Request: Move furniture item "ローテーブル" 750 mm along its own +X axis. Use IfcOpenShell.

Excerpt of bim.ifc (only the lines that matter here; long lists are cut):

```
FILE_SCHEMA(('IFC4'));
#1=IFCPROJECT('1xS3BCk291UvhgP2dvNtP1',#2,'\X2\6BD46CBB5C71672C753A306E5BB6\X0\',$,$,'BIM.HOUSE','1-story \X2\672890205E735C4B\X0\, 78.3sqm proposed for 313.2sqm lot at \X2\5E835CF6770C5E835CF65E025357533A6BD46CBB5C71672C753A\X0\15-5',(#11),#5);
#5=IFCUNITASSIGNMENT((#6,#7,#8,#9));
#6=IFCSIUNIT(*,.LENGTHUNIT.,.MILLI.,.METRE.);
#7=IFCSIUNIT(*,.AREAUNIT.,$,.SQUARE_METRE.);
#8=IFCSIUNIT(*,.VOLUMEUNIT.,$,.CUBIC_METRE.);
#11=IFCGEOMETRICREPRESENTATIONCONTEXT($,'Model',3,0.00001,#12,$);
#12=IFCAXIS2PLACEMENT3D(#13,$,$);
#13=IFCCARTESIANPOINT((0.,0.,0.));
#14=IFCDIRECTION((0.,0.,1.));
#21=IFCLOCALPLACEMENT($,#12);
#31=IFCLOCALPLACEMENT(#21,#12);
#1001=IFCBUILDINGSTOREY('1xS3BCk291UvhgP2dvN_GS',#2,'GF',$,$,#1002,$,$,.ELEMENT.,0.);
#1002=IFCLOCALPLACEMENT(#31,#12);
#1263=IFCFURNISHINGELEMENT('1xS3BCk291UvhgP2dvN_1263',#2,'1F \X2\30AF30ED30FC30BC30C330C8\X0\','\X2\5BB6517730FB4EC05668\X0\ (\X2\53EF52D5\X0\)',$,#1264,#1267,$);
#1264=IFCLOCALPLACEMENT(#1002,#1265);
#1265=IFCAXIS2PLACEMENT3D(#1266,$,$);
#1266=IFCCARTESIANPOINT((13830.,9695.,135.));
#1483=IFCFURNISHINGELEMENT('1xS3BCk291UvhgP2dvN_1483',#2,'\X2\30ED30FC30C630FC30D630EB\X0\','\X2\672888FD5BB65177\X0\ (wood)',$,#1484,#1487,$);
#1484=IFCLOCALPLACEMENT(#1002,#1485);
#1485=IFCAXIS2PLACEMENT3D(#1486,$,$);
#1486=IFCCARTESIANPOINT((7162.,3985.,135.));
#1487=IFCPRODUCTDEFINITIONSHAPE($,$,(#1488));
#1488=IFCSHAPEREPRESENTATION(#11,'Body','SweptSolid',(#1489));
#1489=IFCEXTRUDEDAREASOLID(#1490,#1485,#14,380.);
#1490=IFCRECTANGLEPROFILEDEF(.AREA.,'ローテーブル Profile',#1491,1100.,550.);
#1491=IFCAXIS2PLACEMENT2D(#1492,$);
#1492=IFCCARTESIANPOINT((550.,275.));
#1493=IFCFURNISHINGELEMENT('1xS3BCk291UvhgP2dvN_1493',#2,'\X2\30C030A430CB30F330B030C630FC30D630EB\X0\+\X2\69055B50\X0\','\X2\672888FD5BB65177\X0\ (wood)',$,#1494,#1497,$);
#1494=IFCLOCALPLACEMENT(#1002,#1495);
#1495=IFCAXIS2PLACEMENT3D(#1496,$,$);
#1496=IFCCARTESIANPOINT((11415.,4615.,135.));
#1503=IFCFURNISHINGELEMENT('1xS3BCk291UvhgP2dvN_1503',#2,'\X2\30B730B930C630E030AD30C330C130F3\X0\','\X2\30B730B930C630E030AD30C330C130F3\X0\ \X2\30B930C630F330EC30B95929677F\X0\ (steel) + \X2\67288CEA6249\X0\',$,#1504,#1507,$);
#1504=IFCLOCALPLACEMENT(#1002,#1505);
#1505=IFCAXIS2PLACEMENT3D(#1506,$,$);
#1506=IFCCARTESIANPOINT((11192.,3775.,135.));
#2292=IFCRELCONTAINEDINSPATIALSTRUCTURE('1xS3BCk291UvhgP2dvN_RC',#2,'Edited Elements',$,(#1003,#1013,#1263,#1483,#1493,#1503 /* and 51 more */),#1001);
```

```python
import ifcopenshell
import ifcopenshell.api.geometry
import ifcopenshell.util.placement
import ifcopenshell.util.unit

model = ifcopenshell.open("bim.ifc")
unit_scale = ifcopenshell.util.unit.calculate_unit_scale(model)

item = model.by_guid("1xS3BCk291UvhgP2dvN_1483")
matrix = ifcopenshell.util.placement.get_local_placement(item.ObjectPlacement)
matrix[:3, 3] += matrix[:3, 0] * 0.75 / unit_scale
ifcopenshell.api.geometry.edit_object_placement(model, product=item, matrix=matrix, is_si=False)

print(ifcopenshell.util.placement.get_local_placement(item.ObjectPlacement).round(3) + 0.0)

model.write("bim-out.ifc")
```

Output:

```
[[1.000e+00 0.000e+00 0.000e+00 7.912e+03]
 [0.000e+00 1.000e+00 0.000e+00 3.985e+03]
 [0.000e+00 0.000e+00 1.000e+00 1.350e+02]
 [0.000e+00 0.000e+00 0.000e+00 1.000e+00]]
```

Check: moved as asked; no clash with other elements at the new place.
